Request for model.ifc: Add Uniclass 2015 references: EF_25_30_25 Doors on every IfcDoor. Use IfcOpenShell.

First a look at what the model holds.

```python
import ifcopenshell

model = ifcopenshell.open("model.ifc")
print(model.schema)
print("classifications:", [c.Name for c in model.by_type("IfcClassification")])
for ifc_class in ("IfcDoor", "IfcRoof", "IfcStair", "IfcWall", "IfcWindow"):
    print(ifc_class, len(model.by_type(ifc_class)))
```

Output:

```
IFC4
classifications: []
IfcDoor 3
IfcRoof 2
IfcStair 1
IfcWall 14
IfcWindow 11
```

```python
import ifcopenshell
import ifcopenshell.api.classification

model = ifcopenshell.open("model.ifc")

system = ifcopenshell.api.classification.add_classification(model, classification="Uniclass 2015")

codes = {
    "IfcDoor": ("EF_25_30_25", "Doors"),
}
for ifc_class, (code, name) in codes.items():
    products = model.by_type(ifc_class)
    ifcopenshell.api.classification.add_reference(
        model, products=products, classification=system, identification=code, name=name
    )
    print(code, len(products))

model.write("model_v2.ifc")
```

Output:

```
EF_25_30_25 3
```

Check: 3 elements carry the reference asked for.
